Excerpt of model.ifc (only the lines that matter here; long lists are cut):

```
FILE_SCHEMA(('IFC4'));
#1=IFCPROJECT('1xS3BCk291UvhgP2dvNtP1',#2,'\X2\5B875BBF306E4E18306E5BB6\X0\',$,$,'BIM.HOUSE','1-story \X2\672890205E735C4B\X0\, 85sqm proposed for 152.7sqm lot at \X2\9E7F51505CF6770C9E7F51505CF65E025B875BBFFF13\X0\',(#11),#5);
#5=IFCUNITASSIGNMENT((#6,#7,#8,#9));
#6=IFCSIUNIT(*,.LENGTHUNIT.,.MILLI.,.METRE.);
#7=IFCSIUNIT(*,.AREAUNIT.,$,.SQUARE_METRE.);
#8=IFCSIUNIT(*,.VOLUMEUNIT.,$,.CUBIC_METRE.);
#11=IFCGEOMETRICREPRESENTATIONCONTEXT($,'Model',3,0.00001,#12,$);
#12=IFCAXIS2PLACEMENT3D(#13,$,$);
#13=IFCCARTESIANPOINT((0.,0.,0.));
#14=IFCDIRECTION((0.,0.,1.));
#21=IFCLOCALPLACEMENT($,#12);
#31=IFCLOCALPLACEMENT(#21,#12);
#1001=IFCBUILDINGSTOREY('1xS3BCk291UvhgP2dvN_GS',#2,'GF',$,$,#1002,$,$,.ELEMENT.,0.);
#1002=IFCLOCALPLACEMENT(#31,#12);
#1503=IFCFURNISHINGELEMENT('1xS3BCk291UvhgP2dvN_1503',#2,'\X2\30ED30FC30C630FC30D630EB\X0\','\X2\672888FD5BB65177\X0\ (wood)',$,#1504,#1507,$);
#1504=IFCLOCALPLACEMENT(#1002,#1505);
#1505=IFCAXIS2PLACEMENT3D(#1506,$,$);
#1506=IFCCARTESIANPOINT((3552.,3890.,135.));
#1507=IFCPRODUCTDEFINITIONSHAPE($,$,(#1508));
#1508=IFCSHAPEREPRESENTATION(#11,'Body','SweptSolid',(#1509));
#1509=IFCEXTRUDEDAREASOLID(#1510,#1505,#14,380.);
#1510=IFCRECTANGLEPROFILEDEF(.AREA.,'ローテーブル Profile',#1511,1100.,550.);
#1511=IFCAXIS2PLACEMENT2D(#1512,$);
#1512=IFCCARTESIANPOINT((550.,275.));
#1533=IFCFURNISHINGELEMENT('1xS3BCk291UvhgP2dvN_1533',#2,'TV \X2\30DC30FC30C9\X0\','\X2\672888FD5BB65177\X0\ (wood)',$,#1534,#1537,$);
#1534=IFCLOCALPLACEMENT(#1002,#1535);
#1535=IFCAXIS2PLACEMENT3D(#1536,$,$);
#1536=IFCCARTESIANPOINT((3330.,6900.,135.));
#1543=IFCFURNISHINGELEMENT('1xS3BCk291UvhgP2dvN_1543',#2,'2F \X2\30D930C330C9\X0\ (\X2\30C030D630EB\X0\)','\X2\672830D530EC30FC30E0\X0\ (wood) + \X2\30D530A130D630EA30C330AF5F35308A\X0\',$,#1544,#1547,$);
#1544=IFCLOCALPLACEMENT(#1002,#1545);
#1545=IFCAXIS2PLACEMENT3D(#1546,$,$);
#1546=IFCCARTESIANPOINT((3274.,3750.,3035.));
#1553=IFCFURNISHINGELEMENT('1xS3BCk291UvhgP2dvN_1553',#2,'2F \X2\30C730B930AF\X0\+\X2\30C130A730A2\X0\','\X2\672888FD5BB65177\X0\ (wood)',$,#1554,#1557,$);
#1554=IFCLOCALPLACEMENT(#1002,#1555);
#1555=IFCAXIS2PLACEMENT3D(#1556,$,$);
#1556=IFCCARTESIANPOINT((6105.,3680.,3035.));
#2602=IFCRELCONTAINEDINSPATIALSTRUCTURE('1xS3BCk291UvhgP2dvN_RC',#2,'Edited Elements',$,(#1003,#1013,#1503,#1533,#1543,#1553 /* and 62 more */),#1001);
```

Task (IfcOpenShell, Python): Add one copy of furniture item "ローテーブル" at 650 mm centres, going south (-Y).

```python
import numpy as np
import ifcopenshell
import ifcopenshell.api.geometry
import ifcopenshell.api.root
import ifcopenshell.util.element
import ifcopenshell.util.placement

model = ifcopenshell.open("model.ifc")


def reuse_history(source, copy):
    """copy_class also copies each property set's owner history, people and application; keep the originals."""
    for rel in copy.IsDefinedBy:
        if rel.is_a("IfcRelDefinesByProperties") and (history := rel.RelatingPropertyDefinition.OwnerHistory):
            rel.RelatingPropertyDefinition.OwnerHistory = source.OwnerHistory
            ifcopenshell.util.element.remove_deep2(model, history)


source = model.by_guid("1xS3BCk291UvhgP2dvN_1503")
base = ifcopenshell.util.placement.get_local_placement(source.ObjectPlacement)
step = np.array([0.0, -1.0, 0.0]) * 650.0

for i in range(1, 2):
    copy = ifcopenshell.api.root.copy_class(model, product=source)
    copy.Representation = ifcopenshell.util.element.copy_deep(
        model, source.Representation, exclude=["IfcGeometricRepresentationContext", "IfcRepresentationMap"]
    )
    reuse_history(source, copy)
    matrix = base.copy()
    matrix[:3, 3] += i * step
    print("added at", matrix[:3, 3].round(3) + 0.0)
    ifcopenshell.api.geometry.edit_object_placement(model, product=copy, matrix=matrix, is_si=False)

model.write("model-out.ifc")
```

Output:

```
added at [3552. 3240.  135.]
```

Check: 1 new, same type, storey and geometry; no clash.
